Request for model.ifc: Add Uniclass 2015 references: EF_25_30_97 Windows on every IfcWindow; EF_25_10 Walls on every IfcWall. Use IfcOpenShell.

First a look at what the model holds.

```python
import ifcopenshell

model = ifcopenshell.open("model.ifc")
print(model.schema)
print("classifications:", [c.Name for c in model.by_type("IfcClassification")])
for ifc_class in ("IfcDoor", "IfcRoof", "IfcStair", "IfcWall", "IfcWindow"):
    print(ifc_class, len(model.by_type(ifc_class)))
```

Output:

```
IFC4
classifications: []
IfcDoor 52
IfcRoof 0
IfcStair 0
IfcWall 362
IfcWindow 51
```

```python
import ifcopenshell
import ifcopenshell.api.classification

model = ifcopenshell.open("model.ifc")

system = ifcopenshell.api.classification.add_classification(model, classification="Uniclass 2015")

codes = {
    "IfcWindow": ("EF_25_30_97", "Windows"),
    "IfcWall": ("EF_25_10", "Walls"),
}
for ifc_class, (code, name) in codes.items():
    products = model.by_type(ifc_class)
    ifcopenshell.api.classification.add_reference(
        model, products=products, classification=system, identification=code, name=name
    )
    print(code, len(products))

model.write("model-out.ifc")
```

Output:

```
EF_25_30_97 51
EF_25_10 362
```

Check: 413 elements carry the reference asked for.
